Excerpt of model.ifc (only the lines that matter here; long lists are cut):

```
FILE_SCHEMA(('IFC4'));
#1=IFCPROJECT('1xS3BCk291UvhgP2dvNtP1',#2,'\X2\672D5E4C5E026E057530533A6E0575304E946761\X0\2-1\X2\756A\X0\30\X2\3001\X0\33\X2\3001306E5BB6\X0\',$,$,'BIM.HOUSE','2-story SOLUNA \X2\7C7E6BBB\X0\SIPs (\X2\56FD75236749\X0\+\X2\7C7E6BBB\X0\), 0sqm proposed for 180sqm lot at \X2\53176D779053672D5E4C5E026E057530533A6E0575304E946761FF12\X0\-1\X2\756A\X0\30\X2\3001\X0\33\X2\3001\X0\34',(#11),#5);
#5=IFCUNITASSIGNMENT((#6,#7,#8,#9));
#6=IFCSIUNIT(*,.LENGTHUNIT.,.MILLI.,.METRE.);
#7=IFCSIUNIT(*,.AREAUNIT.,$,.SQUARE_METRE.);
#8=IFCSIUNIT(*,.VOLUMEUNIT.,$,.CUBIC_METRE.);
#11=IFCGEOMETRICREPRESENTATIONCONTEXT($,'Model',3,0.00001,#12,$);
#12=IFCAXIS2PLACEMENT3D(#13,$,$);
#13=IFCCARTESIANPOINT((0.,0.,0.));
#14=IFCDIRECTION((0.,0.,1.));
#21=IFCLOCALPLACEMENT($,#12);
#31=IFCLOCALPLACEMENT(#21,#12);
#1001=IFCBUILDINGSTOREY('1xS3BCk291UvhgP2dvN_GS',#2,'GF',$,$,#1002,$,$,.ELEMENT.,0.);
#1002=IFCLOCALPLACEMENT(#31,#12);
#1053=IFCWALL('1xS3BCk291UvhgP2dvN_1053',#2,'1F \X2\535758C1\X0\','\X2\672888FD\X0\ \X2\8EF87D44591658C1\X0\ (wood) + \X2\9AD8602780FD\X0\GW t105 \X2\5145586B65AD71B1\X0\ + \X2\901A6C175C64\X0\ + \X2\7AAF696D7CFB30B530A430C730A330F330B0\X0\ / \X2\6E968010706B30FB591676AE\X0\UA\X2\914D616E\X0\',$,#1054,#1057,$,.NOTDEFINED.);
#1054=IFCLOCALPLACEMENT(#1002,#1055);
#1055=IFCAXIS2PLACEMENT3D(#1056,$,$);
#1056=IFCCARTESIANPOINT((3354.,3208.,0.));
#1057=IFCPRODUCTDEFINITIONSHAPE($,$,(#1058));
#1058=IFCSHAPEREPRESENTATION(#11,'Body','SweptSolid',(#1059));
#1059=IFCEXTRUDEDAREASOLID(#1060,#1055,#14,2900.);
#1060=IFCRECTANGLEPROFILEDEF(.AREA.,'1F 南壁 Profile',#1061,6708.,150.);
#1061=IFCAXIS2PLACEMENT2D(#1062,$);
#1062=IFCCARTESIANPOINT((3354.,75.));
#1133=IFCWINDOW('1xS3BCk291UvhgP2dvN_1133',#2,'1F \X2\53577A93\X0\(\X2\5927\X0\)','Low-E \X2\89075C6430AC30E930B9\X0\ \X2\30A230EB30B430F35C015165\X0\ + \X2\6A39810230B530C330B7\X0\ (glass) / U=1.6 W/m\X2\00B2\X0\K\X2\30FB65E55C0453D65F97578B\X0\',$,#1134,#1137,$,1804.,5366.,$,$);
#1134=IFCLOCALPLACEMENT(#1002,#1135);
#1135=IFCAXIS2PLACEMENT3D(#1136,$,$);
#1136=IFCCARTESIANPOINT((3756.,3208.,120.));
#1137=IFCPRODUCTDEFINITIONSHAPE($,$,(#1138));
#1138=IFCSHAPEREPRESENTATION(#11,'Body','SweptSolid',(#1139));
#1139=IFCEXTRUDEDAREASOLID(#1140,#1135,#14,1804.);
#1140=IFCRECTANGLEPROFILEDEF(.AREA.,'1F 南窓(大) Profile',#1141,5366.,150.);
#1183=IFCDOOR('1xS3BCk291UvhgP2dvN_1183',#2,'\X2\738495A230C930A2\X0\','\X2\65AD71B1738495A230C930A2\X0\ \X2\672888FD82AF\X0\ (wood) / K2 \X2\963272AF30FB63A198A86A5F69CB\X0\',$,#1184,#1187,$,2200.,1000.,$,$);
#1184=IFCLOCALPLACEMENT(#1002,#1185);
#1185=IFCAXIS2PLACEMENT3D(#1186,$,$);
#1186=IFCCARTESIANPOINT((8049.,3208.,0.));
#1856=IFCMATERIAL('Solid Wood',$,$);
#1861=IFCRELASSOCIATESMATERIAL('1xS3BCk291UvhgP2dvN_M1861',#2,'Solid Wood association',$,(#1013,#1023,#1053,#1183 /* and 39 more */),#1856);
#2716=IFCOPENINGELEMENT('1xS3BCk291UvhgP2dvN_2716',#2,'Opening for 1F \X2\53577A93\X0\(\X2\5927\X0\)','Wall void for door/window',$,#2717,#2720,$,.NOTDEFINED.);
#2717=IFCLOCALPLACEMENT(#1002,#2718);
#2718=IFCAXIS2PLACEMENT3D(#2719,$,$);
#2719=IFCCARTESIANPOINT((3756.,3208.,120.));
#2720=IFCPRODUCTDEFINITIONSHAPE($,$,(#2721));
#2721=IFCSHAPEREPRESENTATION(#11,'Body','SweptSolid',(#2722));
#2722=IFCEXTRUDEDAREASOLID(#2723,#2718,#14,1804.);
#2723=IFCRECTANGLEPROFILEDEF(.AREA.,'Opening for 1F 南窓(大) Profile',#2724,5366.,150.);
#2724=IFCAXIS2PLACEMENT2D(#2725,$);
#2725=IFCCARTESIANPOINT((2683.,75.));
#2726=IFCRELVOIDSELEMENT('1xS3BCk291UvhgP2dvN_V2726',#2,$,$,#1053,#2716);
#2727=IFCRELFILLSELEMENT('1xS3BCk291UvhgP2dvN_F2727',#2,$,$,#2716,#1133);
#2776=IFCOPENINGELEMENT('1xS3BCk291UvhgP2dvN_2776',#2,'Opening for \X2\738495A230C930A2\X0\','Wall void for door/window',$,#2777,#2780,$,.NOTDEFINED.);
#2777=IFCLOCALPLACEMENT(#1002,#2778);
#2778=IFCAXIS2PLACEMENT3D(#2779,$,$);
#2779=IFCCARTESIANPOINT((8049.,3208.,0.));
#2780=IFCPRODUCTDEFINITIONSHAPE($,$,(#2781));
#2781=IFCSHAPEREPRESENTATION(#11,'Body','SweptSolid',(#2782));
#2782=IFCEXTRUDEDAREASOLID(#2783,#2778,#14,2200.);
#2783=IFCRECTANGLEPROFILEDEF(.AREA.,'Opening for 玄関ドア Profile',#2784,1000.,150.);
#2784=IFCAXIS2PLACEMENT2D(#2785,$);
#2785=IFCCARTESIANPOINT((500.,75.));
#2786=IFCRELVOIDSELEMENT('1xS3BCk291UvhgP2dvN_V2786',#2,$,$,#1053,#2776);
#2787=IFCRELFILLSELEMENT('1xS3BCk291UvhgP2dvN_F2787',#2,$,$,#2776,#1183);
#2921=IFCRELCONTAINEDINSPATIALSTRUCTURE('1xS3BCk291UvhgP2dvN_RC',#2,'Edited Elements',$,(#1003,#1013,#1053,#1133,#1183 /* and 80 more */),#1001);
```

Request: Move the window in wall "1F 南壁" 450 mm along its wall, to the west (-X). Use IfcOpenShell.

```python
import ifcopenshell
import ifcopenshell.api.geometry
import ifcopenshell.util.placement
import ifcopenshell.util.unit

model = ifcopenshell.open("model.ifc")
unit_scale = ifcopenshell.util.unit.calculate_unit_scale(model)

window = model.by_guid("1xS3BCk291UvhgP2dvN_1133")
opening = window.FillsVoids[0].RelatingOpeningElement
wall = opening.VoidsElements[0].RelatingBuildingElement

wall_matrix = ifcopenshell.util.placement.get_local_placement(wall.ObjectPlacement)
shift = wall_matrix[:3, 0] * -0.45 / unit_scale
before = ifcopenshell.util.placement.get_local_placement(window.ObjectPlacement)[:3, 3].copy()

# The window is not placed relative to its opening, so move both.
for product in (opening, window):
    matrix = ifcopenshell.util.placement.get_local_placement(product.ObjectPlacement)
    matrix[:3, 3] += shift
    ifcopenshell.api.geometry.edit_object_placement(model, product=product, matrix=matrix, is_si=False)

after = ifcopenshell.util.placement.get_local_placement(window.ObjectPlacement)[:3, 3]
print("window moved by", (after - before).round(3) + 0.0)

model.write("model_rev.ifc")
```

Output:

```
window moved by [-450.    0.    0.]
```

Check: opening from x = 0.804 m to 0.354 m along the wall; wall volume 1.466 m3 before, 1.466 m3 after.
